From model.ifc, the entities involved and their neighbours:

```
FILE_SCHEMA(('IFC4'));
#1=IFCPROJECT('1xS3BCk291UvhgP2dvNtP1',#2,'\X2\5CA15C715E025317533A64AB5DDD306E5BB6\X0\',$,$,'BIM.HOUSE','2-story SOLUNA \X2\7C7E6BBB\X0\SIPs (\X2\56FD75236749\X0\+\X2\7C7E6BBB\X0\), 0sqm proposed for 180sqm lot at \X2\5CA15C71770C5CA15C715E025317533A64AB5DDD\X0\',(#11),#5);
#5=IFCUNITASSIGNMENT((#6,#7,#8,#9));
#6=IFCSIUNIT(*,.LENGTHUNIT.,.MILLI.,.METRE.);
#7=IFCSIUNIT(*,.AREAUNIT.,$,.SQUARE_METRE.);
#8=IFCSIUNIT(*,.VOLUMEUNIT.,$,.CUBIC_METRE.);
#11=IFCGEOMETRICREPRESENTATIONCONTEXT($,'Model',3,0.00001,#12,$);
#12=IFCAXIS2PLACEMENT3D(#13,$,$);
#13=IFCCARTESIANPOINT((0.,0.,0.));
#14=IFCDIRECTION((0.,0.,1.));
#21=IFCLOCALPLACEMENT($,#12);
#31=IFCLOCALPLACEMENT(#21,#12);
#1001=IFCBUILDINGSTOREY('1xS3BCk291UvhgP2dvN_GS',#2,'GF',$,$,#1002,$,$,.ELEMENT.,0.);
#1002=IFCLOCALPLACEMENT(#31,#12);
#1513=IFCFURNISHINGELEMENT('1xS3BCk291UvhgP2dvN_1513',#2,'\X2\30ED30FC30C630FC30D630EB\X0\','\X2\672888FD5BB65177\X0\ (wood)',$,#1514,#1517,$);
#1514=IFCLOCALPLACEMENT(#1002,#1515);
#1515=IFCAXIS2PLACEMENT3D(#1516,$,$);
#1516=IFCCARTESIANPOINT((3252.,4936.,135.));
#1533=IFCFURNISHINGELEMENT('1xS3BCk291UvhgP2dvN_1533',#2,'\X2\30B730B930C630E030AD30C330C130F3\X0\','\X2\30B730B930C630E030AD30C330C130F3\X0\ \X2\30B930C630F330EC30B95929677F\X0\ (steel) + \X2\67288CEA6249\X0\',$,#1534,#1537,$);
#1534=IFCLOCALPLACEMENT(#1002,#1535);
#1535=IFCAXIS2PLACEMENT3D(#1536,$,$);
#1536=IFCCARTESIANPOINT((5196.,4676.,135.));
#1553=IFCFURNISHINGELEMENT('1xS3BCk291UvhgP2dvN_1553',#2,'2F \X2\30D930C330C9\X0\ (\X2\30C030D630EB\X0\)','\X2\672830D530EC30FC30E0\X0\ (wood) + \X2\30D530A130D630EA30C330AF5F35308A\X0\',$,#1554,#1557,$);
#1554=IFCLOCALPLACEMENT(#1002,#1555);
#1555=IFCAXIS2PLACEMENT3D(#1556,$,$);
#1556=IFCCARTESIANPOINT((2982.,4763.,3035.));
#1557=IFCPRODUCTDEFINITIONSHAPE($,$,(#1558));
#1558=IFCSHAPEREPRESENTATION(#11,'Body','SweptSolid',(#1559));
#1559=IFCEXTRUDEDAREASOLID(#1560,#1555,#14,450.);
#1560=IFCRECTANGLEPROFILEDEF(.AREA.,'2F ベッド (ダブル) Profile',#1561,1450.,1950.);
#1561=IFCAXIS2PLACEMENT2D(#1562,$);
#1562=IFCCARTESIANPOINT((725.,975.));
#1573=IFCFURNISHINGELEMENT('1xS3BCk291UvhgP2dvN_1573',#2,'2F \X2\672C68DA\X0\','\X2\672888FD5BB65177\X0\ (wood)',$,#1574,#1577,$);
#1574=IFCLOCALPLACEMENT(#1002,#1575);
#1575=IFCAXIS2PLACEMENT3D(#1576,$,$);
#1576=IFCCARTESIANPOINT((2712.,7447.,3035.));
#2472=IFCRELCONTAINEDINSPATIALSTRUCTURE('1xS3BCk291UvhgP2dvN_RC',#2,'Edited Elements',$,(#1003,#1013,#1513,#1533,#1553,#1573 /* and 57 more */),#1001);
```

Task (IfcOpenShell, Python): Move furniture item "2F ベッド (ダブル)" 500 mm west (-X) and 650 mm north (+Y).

```python
import ifcopenshell
import ifcopenshell.api.geometry
import ifcopenshell.util.placement

model = ifcopenshell.open("model.ifc")

item = model.by_guid("1xS3BCk291UvhgP2dvN_1553")
matrix = ifcopenshell.util.placement.get_local_placement(item.ObjectPlacement)
matrix[0, 3] -= 500.0
matrix[1, 3] += 650.0
ifcopenshell.api.geometry.edit_object_placement(model, product=item, matrix=matrix, is_si=False)

print(ifcopenshell.util.placement.get_local_placement(item.ObjectPlacement).round(3) + 0.0)

model.write("model_updated.ifc")
```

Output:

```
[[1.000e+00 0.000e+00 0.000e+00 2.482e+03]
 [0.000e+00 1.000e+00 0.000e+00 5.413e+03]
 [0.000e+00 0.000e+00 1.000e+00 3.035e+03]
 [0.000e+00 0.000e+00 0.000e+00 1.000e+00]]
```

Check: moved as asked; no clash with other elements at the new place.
